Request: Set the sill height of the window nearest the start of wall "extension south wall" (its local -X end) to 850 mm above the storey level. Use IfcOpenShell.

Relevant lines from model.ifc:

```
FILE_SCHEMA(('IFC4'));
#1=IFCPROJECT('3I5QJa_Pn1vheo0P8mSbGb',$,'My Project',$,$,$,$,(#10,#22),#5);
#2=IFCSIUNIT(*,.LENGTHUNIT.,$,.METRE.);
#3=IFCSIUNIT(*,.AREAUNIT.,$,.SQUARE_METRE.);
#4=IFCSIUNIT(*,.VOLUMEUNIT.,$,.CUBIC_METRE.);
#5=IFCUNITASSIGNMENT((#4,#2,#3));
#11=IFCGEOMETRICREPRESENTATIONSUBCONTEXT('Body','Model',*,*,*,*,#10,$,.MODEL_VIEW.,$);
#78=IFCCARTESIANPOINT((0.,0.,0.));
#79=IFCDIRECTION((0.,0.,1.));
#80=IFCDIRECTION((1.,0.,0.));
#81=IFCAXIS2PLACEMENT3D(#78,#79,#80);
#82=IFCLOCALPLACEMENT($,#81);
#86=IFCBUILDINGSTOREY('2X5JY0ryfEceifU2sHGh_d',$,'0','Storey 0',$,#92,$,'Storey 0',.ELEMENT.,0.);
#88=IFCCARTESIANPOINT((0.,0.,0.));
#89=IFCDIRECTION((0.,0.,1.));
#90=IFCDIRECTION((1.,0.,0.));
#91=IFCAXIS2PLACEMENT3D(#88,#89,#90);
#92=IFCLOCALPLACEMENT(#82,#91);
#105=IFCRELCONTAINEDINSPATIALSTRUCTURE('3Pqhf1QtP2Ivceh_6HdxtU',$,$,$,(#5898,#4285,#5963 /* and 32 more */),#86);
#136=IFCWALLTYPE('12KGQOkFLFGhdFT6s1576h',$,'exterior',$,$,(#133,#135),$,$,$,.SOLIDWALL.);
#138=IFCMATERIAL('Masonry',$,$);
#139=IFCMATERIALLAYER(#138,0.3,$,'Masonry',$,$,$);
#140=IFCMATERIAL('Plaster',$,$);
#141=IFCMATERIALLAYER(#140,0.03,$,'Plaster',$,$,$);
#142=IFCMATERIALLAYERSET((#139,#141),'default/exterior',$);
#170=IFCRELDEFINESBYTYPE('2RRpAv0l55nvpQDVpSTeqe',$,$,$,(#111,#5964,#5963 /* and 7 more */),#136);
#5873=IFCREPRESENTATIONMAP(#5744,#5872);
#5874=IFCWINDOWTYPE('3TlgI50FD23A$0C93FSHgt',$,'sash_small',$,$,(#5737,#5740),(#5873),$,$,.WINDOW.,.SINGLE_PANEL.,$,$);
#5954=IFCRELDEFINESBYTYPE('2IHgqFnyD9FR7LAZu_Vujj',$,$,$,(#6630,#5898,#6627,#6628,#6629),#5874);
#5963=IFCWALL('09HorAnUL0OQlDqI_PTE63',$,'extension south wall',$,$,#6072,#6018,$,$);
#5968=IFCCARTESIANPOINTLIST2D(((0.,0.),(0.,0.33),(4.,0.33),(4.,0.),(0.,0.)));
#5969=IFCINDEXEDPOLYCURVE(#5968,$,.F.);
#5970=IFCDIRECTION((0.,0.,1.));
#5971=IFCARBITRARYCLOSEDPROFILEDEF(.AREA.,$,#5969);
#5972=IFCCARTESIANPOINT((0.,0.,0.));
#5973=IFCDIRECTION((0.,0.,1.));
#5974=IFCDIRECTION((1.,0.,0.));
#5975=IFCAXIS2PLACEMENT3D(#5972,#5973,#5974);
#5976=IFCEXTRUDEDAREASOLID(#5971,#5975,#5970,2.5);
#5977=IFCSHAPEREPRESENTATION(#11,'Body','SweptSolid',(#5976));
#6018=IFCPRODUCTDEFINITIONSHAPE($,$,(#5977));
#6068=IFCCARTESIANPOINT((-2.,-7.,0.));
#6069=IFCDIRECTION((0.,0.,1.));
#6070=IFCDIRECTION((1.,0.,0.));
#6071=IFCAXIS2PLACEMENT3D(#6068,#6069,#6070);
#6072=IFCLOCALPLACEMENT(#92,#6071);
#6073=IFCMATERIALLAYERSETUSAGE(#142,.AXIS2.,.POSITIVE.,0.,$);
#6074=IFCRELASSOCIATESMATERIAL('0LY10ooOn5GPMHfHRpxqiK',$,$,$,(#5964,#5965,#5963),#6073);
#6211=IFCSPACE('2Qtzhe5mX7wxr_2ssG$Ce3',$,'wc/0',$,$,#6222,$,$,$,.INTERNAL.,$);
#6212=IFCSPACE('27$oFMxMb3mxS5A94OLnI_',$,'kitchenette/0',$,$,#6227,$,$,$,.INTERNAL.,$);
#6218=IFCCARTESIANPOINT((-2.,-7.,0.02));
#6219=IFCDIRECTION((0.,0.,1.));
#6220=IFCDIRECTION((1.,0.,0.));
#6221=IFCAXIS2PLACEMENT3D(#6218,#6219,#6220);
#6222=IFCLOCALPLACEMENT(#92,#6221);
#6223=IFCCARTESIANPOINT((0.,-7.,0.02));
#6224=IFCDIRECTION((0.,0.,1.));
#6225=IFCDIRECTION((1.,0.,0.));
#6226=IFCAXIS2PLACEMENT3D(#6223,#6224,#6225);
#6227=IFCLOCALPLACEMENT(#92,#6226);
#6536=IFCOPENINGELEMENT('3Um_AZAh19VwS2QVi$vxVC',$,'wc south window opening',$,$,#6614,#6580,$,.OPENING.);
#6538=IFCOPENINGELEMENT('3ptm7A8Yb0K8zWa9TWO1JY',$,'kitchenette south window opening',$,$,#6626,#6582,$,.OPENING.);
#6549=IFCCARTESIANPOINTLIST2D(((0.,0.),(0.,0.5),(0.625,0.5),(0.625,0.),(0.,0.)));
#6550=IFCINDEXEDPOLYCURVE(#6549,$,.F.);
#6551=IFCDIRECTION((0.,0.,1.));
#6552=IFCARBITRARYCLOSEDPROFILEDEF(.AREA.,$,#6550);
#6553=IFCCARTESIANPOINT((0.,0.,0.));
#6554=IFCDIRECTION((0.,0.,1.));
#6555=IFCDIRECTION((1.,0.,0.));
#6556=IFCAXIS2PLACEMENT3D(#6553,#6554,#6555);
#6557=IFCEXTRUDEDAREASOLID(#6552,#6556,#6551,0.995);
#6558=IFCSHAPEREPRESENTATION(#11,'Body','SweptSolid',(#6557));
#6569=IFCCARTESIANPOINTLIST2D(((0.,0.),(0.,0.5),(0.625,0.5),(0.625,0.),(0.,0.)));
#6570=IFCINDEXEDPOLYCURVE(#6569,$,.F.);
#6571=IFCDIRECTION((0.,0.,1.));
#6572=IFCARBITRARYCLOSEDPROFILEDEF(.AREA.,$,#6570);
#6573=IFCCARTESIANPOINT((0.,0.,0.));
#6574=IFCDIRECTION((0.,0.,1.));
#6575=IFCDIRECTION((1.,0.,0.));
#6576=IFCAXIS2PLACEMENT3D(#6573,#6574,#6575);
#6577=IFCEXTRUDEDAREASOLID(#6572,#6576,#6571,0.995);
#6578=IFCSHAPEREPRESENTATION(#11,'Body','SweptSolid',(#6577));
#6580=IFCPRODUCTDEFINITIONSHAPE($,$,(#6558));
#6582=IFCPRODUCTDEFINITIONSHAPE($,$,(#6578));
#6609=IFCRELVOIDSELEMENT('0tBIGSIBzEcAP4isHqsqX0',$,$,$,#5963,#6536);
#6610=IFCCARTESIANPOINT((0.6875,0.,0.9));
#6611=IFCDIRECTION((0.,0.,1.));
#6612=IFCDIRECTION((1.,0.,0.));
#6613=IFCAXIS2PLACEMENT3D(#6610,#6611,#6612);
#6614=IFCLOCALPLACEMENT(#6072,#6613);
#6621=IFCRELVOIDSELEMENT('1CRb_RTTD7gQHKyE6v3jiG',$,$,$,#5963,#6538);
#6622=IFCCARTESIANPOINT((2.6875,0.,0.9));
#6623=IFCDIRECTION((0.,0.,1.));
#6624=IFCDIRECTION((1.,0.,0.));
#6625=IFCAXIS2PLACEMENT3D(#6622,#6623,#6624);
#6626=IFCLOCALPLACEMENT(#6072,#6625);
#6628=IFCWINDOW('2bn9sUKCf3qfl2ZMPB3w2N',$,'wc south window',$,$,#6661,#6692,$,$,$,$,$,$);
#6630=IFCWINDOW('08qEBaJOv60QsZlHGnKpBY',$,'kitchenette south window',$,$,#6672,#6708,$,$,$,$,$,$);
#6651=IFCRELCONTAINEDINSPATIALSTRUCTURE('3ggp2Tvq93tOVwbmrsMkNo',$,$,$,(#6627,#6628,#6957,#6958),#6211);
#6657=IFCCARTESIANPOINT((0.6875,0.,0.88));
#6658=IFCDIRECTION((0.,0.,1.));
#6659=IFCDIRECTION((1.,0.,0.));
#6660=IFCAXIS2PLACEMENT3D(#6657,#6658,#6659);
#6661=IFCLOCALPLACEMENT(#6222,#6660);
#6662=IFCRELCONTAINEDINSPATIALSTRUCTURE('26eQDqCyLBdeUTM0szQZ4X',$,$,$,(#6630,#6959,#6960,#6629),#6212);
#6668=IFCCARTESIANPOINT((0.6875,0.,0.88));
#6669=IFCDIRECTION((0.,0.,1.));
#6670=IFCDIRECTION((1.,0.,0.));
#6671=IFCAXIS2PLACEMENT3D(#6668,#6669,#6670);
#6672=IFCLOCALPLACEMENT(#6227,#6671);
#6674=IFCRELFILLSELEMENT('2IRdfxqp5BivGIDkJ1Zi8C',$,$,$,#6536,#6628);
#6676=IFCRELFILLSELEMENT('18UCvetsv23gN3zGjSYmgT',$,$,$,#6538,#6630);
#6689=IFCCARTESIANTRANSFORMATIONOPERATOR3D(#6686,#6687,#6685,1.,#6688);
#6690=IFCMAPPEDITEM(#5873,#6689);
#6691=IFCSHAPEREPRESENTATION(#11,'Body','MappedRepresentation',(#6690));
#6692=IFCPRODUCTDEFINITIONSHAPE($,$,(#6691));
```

```python
import numpy as np
import ifcopenshell
import ifcopenshell.api.geometry
import ifcopenshell.geom
import ifcopenshell.util.element
import ifcopenshell.util.placement
import ifcopenshell.util.shape
import ifcopenshell.util.unit

model = ifcopenshell.open("model.ifc")
unit_scale = ifcopenshell.util.unit.calculate_unit_scale(model)

window = model.by_guid("2bn9sUKCf3qfl2ZMPB3w2N")
opening = window.FillsVoids[0].RelatingOpeningElement
storey = ifcopenshell.util.element.get_container(window, ifc_class="IfcBuildingStorey")
level = ifcopenshell.util.placement.get_local_placement(storey.ObjectPlacement)[2, 3]

# The opening's origin need not be at the sill, so measure its lowest point.
shape = ifcopenshell.geom.create_shape(ifcopenshell.geom.settings(), opening)
bottom = ifcopenshell.util.shape.get_shape_bottom_elevation(shape, shape.geometry) / unit_scale
dz = level + 0.85 / unit_scale - bottom

shift = np.array([0.0, 0.0, dz])
# The window is not placed relative to its opening, so move both.
for product in (opening, window):
    matrix = ifcopenshell.util.placement.get_local_placement(product.ObjectPlacement)
    matrix[:3, 3] += shift
    ifcopenshell.api.geometry.edit_object_placement(model, product=product, matrix=matrix, is_si=False)

print(f"moved by {dz * unit_scale:+.3f} m")

model.write("model_rev.ifc")
```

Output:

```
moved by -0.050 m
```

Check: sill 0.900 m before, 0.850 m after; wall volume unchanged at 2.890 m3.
